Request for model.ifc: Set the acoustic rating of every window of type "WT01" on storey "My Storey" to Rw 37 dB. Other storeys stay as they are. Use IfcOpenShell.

First a look at what the model holds.

```python
import ifcopenshell
import ifcopenshell.util.element

model = ifcopenshell.open("model.ifc")
print(model.schema)
storey = next(s for s in model.by_type("IfcBuildingStorey") if s.Name == "My Storey")
windows = [e for e in ifcopenshell.util.element.get_decomposition(storey) if e.is_a("IfcWindow")]
seen = {}
for e in windows:
    element_type = ifcopenshell.util.element.get_type(e)
    key = (element_type.Name if element_type != e and element_type else None, ifcopenshell.util.element.get_pset(e, "Pset_WindowCommon", "AcousticRating"))
    seen[key] = seen.get(key, 0) + 1
for (name, value), count in sorted(seen.items(), key=str):
    print(count, "x", name, "|", value)
```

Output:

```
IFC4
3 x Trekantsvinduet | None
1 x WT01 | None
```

```python
import ifcopenshell
import ifcopenshell.api.pset
import ifcopenshell.util.element

model = ifcopenshell.open("model.ifc")

storey = next(s for s in model.by_type("IfcBuildingStorey") if s.Name == "My Storey")
windows = [e for e in ifcopenshell.util.element.get_decomposition(storey) if e.is_a("IfcWindow")]

count = 0
for e in windows:
    element_type = ifcopenshell.util.element.get_type(e)
    if element_type in (None, e) or element_type.Name != "WT01":
        continue
    # add_pset returns the element's existing set when there is one.
    pset = ifcopenshell.api.pset.add_pset(model, product=e, name="Pset_WindowCommon")
    ifcopenshell.api.pset.edit_pset(model, pset=pset, properties={"AcousticRating": "Rw 37 dB"})
    count += 1

print(count, "windows updated")

model.write("model-out.ifc")
```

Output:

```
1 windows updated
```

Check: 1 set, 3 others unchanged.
